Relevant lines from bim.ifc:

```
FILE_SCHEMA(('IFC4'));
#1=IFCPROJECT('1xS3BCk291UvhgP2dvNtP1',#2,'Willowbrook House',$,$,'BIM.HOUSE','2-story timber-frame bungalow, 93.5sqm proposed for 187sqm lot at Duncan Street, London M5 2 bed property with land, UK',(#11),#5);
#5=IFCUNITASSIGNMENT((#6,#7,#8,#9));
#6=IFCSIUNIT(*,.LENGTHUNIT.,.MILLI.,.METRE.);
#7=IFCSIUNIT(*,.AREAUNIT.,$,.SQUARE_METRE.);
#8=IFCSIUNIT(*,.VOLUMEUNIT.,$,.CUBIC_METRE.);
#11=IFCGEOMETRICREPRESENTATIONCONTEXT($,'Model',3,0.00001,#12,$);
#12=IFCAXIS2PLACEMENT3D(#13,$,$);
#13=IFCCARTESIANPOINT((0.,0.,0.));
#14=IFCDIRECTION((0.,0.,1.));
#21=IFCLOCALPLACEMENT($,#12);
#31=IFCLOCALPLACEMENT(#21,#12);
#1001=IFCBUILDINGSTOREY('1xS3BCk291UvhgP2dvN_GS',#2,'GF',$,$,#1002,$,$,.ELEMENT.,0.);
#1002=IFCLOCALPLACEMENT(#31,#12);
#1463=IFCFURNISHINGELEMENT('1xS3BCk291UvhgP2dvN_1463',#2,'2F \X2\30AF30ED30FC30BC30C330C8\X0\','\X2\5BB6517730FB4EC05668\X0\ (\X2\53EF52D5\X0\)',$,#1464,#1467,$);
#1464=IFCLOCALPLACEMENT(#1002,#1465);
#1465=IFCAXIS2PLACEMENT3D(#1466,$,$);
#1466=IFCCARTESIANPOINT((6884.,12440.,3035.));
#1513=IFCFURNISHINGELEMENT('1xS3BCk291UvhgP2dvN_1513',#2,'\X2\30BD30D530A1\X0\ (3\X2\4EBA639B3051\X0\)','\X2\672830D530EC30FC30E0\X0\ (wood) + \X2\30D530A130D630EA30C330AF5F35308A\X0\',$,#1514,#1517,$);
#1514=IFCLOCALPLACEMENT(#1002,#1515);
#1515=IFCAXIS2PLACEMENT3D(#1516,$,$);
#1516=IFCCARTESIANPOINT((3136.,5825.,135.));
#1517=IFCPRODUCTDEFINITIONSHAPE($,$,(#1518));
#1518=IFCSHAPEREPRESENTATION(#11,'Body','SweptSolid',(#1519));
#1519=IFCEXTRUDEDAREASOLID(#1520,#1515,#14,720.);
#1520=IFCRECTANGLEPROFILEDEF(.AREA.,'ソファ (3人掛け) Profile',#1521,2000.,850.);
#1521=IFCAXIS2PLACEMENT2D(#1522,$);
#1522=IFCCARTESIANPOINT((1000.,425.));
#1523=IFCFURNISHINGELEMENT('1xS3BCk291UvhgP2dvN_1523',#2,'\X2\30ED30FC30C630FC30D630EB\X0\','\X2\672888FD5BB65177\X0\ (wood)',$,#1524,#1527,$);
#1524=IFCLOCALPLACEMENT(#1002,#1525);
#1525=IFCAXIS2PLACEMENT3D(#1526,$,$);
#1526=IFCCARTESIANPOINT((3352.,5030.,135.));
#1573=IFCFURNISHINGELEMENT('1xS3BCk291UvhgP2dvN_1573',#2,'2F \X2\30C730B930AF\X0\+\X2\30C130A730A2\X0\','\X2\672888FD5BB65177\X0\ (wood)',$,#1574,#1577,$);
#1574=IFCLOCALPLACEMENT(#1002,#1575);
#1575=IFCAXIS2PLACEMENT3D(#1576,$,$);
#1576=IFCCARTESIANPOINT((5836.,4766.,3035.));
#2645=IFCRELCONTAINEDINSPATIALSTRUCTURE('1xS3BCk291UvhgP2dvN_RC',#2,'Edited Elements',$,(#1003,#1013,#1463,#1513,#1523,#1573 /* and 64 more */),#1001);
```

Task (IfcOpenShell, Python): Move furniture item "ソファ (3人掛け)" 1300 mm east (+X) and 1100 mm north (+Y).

```python
import ifcopenshell
import ifcopenshell.api.geometry
import ifcopenshell.util.placement

model = ifcopenshell.open("bim.ifc")

item = model.by_guid("1xS3BCk291UvhgP2dvN_1513")
matrix = ifcopenshell.util.placement.get_local_placement(item.ObjectPlacement)
matrix[0, 3] += 1300.0
matrix[1, 3] += 1100.0
ifcopenshell.api.geometry.edit_object_placement(model, product=item, matrix=matrix, is_si=False)

print(ifcopenshell.util.placement.get_local_placement(item.ObjectPlacement).round(3) + 0.0)

model.write("bim_updated.ifc")
```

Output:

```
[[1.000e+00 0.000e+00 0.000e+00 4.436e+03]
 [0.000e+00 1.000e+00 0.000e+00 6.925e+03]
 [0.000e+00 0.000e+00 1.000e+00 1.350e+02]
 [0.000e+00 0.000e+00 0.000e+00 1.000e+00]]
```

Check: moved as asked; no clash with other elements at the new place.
